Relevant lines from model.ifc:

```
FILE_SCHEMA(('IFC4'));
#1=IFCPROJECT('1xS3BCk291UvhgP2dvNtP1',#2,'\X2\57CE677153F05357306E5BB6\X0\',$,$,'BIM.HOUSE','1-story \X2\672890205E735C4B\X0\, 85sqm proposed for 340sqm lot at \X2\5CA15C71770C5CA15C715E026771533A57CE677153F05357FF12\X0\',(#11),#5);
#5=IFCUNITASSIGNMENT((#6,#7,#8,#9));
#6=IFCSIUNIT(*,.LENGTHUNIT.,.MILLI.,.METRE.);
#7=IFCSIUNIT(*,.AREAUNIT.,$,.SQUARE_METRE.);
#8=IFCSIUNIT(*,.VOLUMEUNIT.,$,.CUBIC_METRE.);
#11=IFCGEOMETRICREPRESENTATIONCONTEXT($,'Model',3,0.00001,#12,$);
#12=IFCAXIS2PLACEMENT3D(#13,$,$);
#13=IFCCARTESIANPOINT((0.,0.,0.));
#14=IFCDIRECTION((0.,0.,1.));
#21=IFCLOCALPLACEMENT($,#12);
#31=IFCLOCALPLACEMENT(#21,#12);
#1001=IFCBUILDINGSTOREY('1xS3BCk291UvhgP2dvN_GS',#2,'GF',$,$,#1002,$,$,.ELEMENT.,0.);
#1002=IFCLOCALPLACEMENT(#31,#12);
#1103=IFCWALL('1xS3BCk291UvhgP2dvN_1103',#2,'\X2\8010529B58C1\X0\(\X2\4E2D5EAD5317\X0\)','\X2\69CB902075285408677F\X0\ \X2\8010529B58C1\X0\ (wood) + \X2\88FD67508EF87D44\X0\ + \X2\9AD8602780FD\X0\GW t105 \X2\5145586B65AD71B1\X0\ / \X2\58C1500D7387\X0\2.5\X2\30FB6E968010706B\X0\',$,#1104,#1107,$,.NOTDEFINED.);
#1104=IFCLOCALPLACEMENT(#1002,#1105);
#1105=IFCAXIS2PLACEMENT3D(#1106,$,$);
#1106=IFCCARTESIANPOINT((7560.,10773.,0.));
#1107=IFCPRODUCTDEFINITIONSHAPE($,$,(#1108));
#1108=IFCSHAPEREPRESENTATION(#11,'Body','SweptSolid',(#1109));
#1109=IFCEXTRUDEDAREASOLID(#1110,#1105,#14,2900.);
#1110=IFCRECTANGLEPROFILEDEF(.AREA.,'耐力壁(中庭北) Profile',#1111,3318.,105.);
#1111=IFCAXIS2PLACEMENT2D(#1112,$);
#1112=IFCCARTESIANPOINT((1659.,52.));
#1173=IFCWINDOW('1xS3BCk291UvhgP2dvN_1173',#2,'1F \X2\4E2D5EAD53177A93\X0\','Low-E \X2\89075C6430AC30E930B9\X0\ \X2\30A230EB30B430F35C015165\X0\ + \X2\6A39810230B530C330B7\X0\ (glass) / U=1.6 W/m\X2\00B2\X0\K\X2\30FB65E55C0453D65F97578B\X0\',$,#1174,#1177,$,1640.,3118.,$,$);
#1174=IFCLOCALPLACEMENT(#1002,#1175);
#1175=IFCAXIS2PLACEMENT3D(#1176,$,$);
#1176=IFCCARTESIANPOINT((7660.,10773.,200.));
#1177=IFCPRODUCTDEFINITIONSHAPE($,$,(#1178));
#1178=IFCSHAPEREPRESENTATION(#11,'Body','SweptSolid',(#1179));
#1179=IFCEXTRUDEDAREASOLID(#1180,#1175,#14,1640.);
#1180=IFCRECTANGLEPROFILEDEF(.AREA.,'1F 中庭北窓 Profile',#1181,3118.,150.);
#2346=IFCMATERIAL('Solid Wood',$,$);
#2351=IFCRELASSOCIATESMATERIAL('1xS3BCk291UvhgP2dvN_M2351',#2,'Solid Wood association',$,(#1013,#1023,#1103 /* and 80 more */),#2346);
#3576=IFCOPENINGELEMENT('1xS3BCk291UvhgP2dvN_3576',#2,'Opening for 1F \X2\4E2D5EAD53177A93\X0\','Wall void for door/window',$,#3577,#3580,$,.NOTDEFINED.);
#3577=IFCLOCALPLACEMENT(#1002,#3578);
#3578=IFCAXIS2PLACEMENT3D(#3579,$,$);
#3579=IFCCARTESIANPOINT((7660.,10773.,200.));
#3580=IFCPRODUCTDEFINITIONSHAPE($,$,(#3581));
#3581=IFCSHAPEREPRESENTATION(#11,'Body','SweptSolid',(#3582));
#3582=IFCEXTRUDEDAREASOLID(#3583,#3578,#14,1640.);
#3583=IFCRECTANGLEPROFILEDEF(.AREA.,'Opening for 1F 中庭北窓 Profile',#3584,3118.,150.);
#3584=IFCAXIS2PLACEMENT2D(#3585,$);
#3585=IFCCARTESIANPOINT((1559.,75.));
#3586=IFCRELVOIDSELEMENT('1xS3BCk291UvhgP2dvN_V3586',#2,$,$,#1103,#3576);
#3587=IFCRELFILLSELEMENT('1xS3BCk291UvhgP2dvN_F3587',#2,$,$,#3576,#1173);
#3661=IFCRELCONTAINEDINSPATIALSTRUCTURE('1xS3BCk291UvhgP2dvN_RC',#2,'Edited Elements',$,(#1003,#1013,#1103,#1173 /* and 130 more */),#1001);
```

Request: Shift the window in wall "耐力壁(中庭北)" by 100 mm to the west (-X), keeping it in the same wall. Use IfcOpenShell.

```python
import ifcopenshell
import ifcopenshell.api.geometry
import ifcopenshell.util.placement

model = ifcopenshell.open("model.ifc")

window = model.by_guid("1xS3BCk291UvhgP2dvN_1173")
opening = window.FillsVoids[0].RelatingOpeningElement
wall = opening.VoidsElements[0].RelatingBuildingElement

wall_matrix = ifcopenshell.util.placement.get_local_placement(wall.ObjectPlacement)
shift = wall_matrix[:3, 0] * -100.0
before = ifcopenshell.util.placement.get_local_placement(window.ObjectPlacement)[:3, 3].copy()

# The window is not placed relative to its opening, so move both.
for product in (opening, window):
    matrix = ifcopenshell.util.placement.get_local_placement(product.ObjectPlacement)
    matrix[:3, 3] += shift
    ifcopenshell.api.geometry.edit_object_placement(model, product=product, matrix=matrix, is_si=False)

after = ifcopenshell.util.placement.get_local_placement(window.ObjectPlacement)[:3, 3]
print("window moved by", (after - before).round(3) + 0.0)

model.write("model_edited.ifc")
```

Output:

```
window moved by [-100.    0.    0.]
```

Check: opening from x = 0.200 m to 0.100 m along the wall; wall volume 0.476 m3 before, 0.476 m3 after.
